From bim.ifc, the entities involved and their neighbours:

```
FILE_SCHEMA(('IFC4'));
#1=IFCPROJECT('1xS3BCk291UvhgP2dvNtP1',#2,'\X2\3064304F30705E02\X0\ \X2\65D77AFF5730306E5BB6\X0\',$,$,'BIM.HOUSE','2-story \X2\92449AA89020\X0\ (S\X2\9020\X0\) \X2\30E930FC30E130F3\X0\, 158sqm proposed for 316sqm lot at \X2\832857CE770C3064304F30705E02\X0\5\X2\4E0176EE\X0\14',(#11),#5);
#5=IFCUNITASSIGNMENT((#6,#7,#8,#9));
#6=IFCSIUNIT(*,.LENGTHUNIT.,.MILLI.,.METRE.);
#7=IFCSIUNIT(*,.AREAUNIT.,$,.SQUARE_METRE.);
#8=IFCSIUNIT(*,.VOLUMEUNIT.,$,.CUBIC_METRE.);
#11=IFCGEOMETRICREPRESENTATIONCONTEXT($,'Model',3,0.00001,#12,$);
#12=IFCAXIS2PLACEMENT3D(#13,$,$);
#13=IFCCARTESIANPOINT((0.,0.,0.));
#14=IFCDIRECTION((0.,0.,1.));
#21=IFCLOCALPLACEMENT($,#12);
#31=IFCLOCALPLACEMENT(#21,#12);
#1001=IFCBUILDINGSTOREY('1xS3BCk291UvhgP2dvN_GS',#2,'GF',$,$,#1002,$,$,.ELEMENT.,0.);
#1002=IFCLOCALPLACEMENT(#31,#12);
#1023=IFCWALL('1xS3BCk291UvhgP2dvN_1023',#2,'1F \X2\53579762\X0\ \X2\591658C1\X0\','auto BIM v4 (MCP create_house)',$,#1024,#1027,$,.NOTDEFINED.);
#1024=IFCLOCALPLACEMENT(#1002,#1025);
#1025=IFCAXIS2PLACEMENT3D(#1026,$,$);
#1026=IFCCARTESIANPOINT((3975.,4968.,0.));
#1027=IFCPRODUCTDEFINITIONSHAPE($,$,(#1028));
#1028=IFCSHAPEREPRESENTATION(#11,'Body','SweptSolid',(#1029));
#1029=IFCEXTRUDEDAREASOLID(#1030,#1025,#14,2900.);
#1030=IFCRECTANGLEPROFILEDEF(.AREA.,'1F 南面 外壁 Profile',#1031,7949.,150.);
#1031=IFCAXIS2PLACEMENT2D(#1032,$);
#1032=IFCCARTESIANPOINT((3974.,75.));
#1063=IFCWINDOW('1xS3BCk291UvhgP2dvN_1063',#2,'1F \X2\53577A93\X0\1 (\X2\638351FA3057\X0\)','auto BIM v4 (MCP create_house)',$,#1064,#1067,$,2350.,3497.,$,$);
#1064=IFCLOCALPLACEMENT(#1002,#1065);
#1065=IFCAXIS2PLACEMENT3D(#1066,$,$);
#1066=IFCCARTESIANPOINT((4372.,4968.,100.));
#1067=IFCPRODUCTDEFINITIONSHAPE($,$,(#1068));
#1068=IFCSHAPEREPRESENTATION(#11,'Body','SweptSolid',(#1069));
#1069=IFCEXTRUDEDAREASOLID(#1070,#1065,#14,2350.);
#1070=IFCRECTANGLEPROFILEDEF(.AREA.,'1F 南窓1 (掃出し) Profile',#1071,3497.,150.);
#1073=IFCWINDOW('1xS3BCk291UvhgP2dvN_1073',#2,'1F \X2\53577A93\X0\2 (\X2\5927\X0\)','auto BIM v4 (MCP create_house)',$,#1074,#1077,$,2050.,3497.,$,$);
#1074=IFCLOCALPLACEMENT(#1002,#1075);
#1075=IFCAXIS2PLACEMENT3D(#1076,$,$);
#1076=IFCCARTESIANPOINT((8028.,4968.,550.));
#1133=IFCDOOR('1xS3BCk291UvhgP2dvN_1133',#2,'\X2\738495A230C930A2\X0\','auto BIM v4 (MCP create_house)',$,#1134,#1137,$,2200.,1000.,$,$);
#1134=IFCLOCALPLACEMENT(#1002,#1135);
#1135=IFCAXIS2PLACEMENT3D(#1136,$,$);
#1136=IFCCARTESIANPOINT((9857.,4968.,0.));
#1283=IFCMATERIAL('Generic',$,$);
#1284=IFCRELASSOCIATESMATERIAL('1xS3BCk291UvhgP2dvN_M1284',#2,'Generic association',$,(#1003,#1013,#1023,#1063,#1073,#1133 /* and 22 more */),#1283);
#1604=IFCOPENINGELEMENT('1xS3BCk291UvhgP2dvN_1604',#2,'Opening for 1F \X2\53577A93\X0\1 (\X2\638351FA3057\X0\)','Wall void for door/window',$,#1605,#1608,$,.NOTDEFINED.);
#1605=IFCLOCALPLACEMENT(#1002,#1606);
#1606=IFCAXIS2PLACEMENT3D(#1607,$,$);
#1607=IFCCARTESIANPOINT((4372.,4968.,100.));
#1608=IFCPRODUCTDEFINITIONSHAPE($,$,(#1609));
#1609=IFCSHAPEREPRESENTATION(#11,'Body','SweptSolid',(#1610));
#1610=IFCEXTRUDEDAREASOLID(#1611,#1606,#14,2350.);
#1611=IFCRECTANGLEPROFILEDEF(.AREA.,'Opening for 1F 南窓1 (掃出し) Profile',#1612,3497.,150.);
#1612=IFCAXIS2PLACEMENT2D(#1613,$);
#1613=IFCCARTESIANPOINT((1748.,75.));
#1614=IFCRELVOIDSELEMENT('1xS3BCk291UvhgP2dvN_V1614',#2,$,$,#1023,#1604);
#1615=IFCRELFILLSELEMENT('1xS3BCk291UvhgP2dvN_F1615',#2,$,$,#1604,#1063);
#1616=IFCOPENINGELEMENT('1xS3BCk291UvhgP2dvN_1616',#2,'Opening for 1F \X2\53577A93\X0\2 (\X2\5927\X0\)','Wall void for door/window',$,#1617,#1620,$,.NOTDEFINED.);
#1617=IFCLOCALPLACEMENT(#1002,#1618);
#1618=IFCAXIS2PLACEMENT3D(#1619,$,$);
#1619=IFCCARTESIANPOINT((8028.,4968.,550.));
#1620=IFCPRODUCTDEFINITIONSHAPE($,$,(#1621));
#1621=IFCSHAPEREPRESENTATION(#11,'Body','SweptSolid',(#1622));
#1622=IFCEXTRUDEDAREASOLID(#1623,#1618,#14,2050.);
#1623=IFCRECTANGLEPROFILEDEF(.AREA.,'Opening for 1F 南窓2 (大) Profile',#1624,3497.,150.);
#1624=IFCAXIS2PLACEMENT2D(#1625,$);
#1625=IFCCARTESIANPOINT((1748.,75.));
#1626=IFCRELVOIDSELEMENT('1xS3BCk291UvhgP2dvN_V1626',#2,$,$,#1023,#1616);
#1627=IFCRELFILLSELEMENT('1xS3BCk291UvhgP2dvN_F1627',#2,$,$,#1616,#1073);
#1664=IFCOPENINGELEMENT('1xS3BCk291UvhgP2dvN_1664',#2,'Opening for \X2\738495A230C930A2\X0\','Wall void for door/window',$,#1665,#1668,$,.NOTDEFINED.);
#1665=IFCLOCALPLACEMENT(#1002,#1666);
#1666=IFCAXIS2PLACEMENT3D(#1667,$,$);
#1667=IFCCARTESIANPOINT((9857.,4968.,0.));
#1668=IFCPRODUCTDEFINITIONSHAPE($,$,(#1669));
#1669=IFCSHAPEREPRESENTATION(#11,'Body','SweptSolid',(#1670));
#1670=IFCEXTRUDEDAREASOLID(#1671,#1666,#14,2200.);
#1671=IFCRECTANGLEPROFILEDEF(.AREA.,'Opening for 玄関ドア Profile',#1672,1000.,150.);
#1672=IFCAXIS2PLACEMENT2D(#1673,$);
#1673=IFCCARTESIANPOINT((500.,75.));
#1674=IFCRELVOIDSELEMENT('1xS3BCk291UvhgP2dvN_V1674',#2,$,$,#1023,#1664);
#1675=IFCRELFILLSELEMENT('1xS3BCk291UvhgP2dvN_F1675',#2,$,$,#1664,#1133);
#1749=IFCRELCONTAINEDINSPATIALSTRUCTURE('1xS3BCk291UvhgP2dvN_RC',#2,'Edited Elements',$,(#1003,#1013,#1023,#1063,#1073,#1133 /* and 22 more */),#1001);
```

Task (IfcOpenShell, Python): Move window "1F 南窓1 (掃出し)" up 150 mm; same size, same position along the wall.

```python
import numpy as np
import ifcopenshell
import ifcopenshell.api.geometry
import ifcopenshell.util.placement
import ifcopenshell.util.unit

model = ifcopenshell.open("bim.ifc")
unit_scale = ifcopenshell.util.unit.calculate_unit_scale(model)

window = model.by_guid("1xS3BCk291UvhgP2dvN_1063")
opening = window.FillsVoids[0].RelatingOpeningElement
dz = 0.15 / unit_scale

shift = np.array([0.0, 0.0, dz])
# The window is not placed relative to its opening, so move both.
for product in (opening, window):
    matrix = ifcopenshell.util.placement.get_local_placement(product.ObjectPlacement)
    matrix[:3, 3] += shift
    ifcopenshell.api.geometry.edit_object_placement(model, product=product, matrix=matrix, is_si=False)

print(f"moved by {dz * unit_scale:+.3f} m")

model.write("bim_rev.ifc")
```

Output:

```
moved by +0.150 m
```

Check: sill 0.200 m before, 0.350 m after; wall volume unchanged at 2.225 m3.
